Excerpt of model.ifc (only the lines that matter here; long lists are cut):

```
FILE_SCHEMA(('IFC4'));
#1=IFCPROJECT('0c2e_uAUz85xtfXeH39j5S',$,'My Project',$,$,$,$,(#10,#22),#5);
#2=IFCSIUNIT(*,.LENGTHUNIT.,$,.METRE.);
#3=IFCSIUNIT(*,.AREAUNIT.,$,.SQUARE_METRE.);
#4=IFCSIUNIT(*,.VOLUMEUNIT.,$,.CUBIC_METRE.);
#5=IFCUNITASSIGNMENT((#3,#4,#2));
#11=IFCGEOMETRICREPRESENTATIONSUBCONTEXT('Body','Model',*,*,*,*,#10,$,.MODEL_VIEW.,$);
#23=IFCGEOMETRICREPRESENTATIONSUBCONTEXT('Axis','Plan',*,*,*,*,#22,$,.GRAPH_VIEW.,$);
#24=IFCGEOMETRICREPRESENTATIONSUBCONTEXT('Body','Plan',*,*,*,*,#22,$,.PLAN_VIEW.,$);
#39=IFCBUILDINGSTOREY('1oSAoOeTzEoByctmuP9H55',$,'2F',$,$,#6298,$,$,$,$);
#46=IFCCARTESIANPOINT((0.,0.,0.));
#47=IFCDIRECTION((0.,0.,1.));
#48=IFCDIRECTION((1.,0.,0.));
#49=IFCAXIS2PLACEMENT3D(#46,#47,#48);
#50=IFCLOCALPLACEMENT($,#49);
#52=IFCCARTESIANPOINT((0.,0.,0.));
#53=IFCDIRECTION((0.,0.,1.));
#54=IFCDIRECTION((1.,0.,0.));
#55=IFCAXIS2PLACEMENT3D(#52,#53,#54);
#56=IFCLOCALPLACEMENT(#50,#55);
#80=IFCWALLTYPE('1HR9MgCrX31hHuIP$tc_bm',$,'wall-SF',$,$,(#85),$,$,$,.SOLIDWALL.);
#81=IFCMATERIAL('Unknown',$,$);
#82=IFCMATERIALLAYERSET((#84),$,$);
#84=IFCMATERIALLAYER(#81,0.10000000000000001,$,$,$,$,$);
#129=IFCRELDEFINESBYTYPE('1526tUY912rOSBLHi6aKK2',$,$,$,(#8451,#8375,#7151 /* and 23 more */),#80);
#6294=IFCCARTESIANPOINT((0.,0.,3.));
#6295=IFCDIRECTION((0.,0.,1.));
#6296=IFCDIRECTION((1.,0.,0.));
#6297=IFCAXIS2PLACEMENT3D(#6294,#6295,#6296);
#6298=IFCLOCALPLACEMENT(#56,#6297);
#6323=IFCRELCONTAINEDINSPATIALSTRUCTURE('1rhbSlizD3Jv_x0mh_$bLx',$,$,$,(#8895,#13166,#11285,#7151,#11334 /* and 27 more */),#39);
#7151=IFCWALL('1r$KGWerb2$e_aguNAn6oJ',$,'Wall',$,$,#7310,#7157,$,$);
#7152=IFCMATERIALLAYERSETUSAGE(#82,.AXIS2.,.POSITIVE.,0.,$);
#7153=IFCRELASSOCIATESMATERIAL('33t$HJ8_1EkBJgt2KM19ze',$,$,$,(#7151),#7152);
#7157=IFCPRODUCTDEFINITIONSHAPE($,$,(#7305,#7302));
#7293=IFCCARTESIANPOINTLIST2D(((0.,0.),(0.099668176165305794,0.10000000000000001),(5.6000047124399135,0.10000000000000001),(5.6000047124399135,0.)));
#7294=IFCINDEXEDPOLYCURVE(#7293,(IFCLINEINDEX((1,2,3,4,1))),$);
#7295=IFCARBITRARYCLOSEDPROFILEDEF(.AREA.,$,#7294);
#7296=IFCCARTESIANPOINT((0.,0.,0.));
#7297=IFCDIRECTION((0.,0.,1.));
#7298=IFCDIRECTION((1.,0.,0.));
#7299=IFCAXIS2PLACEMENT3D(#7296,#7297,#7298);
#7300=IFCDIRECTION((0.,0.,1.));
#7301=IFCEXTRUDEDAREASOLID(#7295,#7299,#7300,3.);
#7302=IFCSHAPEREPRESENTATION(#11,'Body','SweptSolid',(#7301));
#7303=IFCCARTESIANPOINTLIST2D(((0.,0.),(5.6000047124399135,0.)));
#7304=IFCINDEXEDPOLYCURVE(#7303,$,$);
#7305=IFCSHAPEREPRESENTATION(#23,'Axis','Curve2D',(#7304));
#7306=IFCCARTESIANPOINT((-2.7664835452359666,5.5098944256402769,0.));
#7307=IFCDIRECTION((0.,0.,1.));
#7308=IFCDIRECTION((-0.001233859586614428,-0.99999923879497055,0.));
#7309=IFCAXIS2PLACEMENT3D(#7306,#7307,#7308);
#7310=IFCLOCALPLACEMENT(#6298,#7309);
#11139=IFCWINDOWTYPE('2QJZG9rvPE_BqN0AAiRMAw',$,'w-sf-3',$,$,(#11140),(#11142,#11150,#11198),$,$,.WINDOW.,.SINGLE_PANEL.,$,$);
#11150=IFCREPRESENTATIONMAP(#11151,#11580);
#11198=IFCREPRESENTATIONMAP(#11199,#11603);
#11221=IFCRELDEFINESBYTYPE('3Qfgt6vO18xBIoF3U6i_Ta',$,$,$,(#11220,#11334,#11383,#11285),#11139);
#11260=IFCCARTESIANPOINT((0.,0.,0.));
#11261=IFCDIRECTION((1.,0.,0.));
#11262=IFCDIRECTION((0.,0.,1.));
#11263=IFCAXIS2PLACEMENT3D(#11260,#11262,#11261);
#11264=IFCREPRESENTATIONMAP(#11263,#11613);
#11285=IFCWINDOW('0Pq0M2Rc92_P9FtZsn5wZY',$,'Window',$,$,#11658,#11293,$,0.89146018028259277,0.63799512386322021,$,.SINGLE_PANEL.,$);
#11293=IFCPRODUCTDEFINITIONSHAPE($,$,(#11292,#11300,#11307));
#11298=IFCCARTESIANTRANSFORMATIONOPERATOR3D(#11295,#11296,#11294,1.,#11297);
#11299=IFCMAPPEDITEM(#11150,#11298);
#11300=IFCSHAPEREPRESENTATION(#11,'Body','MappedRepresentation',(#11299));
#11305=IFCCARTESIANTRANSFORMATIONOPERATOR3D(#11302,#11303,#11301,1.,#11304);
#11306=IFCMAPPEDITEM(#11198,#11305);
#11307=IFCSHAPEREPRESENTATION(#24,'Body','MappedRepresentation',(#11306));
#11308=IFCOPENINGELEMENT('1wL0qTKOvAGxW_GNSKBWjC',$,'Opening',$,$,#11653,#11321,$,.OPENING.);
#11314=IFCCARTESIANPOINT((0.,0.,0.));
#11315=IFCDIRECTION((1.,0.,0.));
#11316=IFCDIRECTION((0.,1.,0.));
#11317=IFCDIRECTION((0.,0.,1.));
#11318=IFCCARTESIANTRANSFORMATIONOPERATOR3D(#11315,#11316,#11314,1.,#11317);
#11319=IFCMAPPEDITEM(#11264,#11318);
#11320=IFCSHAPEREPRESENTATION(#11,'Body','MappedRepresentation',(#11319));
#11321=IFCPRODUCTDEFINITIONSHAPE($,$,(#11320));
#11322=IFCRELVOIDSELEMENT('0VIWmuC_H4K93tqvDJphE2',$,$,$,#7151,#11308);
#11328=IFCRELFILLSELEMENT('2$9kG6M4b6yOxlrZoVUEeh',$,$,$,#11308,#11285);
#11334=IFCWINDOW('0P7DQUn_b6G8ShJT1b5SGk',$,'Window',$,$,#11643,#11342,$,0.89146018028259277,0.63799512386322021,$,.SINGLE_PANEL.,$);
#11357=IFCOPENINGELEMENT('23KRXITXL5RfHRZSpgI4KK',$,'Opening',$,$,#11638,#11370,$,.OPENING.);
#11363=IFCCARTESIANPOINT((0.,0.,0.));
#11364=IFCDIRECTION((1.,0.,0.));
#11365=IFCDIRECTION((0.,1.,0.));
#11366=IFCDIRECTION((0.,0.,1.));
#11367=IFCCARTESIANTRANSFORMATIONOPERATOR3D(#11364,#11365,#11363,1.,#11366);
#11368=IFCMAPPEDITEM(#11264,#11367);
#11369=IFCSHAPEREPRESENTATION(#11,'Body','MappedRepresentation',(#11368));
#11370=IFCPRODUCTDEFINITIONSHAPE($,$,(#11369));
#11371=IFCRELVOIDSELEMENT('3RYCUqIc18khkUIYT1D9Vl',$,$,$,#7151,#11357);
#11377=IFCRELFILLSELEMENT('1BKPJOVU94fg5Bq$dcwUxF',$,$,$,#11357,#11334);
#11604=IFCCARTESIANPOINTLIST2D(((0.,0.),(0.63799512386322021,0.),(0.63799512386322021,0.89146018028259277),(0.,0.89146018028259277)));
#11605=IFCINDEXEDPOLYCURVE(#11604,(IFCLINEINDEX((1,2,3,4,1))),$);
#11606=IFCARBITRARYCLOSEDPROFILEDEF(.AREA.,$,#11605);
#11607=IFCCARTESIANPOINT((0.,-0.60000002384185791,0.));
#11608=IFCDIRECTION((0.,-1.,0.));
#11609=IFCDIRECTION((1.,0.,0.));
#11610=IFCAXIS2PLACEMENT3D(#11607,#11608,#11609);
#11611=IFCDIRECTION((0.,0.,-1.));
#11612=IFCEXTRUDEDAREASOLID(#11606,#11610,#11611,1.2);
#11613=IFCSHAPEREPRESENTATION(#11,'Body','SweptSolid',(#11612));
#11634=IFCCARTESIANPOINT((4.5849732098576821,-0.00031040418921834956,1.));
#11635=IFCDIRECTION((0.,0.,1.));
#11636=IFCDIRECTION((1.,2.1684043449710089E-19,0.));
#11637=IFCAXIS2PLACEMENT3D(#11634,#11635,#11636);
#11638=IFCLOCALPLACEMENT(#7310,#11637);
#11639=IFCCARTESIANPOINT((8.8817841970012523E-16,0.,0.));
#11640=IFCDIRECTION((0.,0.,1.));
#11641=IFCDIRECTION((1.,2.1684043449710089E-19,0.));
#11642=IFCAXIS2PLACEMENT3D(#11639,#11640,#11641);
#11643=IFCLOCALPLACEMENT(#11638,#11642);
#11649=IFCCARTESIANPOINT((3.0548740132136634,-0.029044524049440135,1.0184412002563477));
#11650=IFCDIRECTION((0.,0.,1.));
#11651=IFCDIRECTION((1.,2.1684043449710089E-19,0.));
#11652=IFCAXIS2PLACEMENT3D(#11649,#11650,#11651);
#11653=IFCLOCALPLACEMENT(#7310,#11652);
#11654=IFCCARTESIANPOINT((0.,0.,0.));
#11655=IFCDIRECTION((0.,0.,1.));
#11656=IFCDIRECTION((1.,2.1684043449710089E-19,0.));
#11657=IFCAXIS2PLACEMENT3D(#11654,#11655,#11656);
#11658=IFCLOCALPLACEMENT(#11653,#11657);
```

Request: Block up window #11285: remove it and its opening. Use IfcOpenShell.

```python
import ifcopenshell
import ifcopenshell.api.feature
import ifcopenshell.api.root
import ifcopenshell.geom
import ifcopenshell.util.shape

model = ifcopenshell.open("model.ifc")
settings = ifcopenshell.geom.settings()


def volume(element):
    """Net volume in cubic metres, openings subtracted."""
    shape = ifcopenshell.geom.create_shape(settings, element)
    return ifcopenshell.util.shape.get_volume(shape.geometry)


window = model.by_guid("0Pq0M2Rc92_P9FtZsn5wZY")
opening = window.FillsVoids[0].RelatingOpeningElement
wall = opening.VoidsElements[0].RelatingBuildingElement
before = volume(wall)

ifcopenshell.api.root.remove_product(model, product=window)
ifcopenshell.api.feature.remove_feature(model, feature=opening)

after = volume(wall)

print(f"wall volume {before:.3f} -> {after:.3f} m3")

model.write("model_rev.ifc")
```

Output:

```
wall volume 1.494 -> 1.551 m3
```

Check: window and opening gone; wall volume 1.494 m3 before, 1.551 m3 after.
